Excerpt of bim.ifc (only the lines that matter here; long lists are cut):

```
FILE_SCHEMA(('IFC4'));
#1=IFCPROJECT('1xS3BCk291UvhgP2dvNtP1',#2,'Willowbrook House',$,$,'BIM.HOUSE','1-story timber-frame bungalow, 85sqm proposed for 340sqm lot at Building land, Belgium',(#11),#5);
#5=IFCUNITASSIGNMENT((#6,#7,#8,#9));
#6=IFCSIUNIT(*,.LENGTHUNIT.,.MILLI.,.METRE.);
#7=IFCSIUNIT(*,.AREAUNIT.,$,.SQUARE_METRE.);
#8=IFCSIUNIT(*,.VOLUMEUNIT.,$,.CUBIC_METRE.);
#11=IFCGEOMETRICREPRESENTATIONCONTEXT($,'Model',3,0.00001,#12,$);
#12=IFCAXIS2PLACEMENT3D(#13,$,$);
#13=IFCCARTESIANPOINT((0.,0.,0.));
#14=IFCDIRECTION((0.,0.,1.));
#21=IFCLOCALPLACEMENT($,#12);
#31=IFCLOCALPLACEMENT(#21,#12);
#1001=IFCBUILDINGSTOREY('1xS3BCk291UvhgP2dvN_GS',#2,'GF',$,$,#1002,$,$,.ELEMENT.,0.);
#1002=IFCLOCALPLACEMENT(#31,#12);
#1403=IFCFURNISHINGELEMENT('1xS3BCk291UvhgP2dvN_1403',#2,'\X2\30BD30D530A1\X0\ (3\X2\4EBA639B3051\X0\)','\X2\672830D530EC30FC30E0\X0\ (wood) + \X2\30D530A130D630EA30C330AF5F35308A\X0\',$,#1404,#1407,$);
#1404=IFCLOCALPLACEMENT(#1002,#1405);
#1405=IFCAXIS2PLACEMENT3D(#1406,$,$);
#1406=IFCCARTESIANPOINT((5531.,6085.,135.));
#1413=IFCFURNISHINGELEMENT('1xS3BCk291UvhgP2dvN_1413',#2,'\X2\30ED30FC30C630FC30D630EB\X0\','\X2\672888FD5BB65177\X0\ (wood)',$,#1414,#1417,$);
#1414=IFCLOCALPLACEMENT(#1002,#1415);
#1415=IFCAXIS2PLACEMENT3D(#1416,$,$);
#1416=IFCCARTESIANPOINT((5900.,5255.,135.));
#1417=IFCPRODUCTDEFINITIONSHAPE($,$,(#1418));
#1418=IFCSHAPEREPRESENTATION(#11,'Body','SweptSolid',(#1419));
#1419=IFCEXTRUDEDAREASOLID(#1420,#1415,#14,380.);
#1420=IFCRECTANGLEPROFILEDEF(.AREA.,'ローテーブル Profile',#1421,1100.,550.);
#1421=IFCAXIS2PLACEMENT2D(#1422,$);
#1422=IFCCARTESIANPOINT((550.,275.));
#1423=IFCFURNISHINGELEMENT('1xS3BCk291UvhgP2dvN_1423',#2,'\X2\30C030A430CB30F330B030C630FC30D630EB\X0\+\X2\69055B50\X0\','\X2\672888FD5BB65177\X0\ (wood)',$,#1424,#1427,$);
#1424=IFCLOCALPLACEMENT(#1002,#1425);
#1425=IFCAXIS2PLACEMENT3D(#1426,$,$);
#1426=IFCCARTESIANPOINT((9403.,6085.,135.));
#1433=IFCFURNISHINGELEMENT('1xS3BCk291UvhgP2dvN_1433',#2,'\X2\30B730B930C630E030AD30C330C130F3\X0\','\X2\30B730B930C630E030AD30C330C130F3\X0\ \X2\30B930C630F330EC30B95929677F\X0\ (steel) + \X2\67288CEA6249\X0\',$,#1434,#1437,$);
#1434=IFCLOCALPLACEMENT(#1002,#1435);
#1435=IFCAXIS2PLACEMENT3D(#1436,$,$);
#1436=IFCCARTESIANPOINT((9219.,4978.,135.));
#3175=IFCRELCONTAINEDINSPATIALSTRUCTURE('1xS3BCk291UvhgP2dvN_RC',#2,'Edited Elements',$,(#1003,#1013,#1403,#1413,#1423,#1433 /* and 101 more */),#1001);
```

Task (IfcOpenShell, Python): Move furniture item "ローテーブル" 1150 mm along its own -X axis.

```python
import ifcopenshell
import ifcopenshell.api.geometry
import ifcopenshell.util.placement
import ifcopenshell.util.unit

model = ifcopenshell.open("bim.ifc")
unit_scale = ifcopenshell.util.unit.calculate_unit_scale(model)

item = model.by_id(1413)
matrix = ifcopenshell.util.placement.get_local_placement(item.ObjectPlacement)
matrix[:3, 3] -= matrix[:3, 0] * 1.15 / unit_scale
ifcopenshell.api.geometry.edit_object_placement(model, product=item, matrix=matrix, is_si=False)

print(ifcopenshell.util.placement.get_local_placement(item.ObjectPlacement).round(3) + 0.0)

model.write("bim_updated.ifc")
```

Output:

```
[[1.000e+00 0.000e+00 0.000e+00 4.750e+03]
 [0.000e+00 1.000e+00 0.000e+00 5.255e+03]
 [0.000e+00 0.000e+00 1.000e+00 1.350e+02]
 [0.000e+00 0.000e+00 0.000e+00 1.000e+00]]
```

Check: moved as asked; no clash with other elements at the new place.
